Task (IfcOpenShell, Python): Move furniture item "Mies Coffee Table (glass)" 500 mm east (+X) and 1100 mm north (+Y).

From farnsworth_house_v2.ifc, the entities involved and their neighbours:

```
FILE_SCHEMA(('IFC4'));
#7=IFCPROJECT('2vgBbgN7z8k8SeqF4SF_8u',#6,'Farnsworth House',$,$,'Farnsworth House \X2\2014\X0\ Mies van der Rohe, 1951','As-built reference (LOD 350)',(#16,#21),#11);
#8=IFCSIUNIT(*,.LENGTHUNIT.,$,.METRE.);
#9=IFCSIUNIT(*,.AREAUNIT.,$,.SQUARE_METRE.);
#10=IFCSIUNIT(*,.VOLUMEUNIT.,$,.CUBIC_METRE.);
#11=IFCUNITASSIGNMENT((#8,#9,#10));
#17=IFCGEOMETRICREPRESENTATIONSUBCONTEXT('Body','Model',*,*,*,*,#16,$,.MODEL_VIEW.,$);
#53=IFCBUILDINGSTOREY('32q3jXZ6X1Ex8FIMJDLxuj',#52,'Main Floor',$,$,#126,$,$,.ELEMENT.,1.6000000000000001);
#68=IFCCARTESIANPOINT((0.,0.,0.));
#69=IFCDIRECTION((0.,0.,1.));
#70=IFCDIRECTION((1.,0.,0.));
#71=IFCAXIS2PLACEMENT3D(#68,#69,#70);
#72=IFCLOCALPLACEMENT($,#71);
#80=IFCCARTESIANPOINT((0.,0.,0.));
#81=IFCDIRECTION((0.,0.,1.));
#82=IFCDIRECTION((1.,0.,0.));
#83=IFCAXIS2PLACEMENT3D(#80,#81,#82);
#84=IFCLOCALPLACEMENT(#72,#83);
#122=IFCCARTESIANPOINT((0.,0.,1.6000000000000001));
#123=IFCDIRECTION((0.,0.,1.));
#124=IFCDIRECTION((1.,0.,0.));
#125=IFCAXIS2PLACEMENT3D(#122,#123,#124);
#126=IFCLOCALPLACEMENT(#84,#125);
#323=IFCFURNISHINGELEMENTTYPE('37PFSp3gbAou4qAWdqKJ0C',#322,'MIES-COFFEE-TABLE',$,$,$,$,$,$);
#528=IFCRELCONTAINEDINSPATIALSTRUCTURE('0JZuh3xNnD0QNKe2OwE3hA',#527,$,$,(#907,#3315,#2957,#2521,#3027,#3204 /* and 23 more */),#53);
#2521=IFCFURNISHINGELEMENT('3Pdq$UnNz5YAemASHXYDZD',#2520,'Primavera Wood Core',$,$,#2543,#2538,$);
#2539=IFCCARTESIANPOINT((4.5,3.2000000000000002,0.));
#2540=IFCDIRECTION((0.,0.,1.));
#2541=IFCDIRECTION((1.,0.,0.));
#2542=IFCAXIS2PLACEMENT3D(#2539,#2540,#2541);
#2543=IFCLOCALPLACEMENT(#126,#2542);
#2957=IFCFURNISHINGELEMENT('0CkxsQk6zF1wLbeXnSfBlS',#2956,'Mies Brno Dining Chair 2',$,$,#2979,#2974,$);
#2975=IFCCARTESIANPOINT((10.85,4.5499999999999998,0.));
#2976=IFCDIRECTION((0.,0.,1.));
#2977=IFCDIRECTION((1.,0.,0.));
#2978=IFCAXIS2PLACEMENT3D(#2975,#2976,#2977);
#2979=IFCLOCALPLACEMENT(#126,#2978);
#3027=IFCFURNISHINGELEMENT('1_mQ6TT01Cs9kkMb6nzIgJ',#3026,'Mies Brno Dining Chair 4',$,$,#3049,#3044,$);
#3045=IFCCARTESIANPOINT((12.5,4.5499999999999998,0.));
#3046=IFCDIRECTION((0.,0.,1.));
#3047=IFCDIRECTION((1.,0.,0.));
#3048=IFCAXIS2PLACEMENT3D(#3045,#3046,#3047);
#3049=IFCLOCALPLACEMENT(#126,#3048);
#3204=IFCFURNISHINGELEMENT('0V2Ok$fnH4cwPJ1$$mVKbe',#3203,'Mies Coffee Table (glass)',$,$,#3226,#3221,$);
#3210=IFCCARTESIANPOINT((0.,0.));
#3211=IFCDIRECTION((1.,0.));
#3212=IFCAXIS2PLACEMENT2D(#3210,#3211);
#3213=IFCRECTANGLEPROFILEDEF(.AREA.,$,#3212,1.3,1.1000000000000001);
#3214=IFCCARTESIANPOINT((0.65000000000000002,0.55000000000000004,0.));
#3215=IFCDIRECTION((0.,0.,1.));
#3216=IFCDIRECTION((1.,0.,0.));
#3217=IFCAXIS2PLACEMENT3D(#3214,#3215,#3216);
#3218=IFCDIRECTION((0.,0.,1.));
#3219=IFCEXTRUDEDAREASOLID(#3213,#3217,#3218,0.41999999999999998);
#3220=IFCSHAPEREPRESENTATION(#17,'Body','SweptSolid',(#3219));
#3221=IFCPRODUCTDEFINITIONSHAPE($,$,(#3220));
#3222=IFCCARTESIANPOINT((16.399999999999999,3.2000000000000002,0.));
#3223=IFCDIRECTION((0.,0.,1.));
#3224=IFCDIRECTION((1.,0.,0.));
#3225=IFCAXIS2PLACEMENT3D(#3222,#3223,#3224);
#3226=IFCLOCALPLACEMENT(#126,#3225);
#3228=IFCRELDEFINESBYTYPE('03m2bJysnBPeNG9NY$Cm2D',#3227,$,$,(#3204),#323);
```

```python
import ifcopenshell
import ifcopenshell.api.geometry
import ifcopenshell.util.placement

model = ifcopenshell.open("farnsworth_house_v2.ifc")

item = model.by_guid("0V2Ok$fnH4cwPJ1$$mVKbe")
matrix = ifcopenshell.util.placement.get_local_placement(item.ObjectPlacement)
matrix[0, 3] += 0.5
matrix[1, 3] += 1.1
ifcopenshell.api.geometry.edit_object_placement(model, product=item, matrix=matrix, is_si=False)

print(ifcopenshell.util.placement.get_local_placement(item.ObjectPlacement).round(3) + 0.0)

model.write("farnsworth_house_v2_edited.ifc")
```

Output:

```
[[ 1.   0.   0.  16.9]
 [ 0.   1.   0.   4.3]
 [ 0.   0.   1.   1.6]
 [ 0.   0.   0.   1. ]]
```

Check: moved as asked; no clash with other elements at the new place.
